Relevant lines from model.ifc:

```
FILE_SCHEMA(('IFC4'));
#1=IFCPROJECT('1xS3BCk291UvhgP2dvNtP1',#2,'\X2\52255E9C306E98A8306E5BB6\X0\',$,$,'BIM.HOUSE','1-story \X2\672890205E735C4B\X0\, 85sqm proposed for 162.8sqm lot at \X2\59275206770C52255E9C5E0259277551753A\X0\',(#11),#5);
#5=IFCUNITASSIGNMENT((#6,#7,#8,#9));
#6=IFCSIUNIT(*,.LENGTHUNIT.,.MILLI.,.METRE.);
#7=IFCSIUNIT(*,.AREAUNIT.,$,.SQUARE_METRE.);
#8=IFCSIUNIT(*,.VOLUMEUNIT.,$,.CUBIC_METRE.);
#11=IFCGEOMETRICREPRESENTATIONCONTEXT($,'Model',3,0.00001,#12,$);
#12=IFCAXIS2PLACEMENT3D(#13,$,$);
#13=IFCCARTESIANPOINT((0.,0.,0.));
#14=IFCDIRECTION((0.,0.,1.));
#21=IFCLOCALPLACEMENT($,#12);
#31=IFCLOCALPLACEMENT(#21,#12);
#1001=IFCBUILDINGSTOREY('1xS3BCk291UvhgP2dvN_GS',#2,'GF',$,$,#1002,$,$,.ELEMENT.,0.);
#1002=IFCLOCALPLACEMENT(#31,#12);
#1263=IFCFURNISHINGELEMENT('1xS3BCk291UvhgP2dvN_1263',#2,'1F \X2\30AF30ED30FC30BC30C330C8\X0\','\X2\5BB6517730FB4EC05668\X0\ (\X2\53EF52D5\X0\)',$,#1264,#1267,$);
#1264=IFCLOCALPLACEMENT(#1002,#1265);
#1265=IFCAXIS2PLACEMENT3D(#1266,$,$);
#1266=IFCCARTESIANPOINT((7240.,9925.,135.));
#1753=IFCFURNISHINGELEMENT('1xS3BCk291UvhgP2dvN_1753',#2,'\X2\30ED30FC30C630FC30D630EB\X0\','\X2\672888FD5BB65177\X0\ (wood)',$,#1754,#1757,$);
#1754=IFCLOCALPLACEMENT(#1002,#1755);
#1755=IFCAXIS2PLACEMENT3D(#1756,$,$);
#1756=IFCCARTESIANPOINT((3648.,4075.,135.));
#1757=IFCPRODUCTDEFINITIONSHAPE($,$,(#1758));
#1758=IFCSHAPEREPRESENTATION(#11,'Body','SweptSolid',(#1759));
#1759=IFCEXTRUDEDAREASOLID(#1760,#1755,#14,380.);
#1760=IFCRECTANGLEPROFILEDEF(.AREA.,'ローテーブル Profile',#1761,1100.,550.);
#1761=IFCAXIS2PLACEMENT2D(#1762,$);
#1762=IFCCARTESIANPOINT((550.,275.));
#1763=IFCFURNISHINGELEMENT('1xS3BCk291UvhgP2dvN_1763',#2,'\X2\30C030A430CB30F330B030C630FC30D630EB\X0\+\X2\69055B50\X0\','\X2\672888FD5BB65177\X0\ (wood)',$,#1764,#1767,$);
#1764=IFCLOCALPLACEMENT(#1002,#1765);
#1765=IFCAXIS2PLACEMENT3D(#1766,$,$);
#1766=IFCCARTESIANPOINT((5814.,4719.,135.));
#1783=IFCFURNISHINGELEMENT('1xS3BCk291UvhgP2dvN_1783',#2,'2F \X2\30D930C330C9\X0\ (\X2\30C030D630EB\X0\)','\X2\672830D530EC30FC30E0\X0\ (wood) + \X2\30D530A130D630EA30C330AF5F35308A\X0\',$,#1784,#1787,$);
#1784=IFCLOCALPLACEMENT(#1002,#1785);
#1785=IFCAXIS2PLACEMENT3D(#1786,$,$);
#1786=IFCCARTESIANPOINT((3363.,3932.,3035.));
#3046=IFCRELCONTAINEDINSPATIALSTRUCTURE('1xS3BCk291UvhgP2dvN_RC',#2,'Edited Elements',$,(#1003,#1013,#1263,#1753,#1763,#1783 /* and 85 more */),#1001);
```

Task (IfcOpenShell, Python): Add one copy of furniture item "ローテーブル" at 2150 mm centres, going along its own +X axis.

```python
import ifcopenshell
import ifcopenshell.api.geometry
import ifcopenshell.api.root
import ifcopenshell.util.element
import ifcopenshell.util.placement
import ifcopenshell.util.unit

model = ifcopenshell.open("model.ifc")
unit_scale = ifcopenshell.util.unit.calculate_unit_scale(model)


def reuse_history(source, copy):
    """copy_class also copies each property set's owner history, people and application; keep the originals."""
    for rel in copy.IsDefinedBy:
        if rel.is_a("IfcRelDefinesByProperties") and (history := rel.RelatingPropertyDefinition.OwnerHistory):
            rel.RelatingPropertyDefinition.OwnerHistory = source.OwnerHistory
            ifcopenshell.util.element.remove_deep2(model, history)


source = model.by_id(1753)
base = ifcopenshell.util.placement.get_local_placement(source.ObjectPlacement)
step = base[:3, 0] * 2.15 / unit_scale

for i in range(1, 2):
    copy = ifcopenshell.api.root.copy_class(model, product=source)
    copy.Representation = ifcopenshell.util.element.copy_deep(
        model, source.Representation, exclude=["IfcGeometricRepresentationContext", "IfcRepresentationMap"]
    )
    reuse_history(source, copy)
    matrix = base.copy()
    matrix[:3, 3] += i * step
    print("added at", matrix[:3, 3].round(3) + 0.0)
    ifcopenshell.api.geometry.edit_object_placement(model, product=copy, matrix=matrix, is_si=False)

model.write("model-out.ifc")
```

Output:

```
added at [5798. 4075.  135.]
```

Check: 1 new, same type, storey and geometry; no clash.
